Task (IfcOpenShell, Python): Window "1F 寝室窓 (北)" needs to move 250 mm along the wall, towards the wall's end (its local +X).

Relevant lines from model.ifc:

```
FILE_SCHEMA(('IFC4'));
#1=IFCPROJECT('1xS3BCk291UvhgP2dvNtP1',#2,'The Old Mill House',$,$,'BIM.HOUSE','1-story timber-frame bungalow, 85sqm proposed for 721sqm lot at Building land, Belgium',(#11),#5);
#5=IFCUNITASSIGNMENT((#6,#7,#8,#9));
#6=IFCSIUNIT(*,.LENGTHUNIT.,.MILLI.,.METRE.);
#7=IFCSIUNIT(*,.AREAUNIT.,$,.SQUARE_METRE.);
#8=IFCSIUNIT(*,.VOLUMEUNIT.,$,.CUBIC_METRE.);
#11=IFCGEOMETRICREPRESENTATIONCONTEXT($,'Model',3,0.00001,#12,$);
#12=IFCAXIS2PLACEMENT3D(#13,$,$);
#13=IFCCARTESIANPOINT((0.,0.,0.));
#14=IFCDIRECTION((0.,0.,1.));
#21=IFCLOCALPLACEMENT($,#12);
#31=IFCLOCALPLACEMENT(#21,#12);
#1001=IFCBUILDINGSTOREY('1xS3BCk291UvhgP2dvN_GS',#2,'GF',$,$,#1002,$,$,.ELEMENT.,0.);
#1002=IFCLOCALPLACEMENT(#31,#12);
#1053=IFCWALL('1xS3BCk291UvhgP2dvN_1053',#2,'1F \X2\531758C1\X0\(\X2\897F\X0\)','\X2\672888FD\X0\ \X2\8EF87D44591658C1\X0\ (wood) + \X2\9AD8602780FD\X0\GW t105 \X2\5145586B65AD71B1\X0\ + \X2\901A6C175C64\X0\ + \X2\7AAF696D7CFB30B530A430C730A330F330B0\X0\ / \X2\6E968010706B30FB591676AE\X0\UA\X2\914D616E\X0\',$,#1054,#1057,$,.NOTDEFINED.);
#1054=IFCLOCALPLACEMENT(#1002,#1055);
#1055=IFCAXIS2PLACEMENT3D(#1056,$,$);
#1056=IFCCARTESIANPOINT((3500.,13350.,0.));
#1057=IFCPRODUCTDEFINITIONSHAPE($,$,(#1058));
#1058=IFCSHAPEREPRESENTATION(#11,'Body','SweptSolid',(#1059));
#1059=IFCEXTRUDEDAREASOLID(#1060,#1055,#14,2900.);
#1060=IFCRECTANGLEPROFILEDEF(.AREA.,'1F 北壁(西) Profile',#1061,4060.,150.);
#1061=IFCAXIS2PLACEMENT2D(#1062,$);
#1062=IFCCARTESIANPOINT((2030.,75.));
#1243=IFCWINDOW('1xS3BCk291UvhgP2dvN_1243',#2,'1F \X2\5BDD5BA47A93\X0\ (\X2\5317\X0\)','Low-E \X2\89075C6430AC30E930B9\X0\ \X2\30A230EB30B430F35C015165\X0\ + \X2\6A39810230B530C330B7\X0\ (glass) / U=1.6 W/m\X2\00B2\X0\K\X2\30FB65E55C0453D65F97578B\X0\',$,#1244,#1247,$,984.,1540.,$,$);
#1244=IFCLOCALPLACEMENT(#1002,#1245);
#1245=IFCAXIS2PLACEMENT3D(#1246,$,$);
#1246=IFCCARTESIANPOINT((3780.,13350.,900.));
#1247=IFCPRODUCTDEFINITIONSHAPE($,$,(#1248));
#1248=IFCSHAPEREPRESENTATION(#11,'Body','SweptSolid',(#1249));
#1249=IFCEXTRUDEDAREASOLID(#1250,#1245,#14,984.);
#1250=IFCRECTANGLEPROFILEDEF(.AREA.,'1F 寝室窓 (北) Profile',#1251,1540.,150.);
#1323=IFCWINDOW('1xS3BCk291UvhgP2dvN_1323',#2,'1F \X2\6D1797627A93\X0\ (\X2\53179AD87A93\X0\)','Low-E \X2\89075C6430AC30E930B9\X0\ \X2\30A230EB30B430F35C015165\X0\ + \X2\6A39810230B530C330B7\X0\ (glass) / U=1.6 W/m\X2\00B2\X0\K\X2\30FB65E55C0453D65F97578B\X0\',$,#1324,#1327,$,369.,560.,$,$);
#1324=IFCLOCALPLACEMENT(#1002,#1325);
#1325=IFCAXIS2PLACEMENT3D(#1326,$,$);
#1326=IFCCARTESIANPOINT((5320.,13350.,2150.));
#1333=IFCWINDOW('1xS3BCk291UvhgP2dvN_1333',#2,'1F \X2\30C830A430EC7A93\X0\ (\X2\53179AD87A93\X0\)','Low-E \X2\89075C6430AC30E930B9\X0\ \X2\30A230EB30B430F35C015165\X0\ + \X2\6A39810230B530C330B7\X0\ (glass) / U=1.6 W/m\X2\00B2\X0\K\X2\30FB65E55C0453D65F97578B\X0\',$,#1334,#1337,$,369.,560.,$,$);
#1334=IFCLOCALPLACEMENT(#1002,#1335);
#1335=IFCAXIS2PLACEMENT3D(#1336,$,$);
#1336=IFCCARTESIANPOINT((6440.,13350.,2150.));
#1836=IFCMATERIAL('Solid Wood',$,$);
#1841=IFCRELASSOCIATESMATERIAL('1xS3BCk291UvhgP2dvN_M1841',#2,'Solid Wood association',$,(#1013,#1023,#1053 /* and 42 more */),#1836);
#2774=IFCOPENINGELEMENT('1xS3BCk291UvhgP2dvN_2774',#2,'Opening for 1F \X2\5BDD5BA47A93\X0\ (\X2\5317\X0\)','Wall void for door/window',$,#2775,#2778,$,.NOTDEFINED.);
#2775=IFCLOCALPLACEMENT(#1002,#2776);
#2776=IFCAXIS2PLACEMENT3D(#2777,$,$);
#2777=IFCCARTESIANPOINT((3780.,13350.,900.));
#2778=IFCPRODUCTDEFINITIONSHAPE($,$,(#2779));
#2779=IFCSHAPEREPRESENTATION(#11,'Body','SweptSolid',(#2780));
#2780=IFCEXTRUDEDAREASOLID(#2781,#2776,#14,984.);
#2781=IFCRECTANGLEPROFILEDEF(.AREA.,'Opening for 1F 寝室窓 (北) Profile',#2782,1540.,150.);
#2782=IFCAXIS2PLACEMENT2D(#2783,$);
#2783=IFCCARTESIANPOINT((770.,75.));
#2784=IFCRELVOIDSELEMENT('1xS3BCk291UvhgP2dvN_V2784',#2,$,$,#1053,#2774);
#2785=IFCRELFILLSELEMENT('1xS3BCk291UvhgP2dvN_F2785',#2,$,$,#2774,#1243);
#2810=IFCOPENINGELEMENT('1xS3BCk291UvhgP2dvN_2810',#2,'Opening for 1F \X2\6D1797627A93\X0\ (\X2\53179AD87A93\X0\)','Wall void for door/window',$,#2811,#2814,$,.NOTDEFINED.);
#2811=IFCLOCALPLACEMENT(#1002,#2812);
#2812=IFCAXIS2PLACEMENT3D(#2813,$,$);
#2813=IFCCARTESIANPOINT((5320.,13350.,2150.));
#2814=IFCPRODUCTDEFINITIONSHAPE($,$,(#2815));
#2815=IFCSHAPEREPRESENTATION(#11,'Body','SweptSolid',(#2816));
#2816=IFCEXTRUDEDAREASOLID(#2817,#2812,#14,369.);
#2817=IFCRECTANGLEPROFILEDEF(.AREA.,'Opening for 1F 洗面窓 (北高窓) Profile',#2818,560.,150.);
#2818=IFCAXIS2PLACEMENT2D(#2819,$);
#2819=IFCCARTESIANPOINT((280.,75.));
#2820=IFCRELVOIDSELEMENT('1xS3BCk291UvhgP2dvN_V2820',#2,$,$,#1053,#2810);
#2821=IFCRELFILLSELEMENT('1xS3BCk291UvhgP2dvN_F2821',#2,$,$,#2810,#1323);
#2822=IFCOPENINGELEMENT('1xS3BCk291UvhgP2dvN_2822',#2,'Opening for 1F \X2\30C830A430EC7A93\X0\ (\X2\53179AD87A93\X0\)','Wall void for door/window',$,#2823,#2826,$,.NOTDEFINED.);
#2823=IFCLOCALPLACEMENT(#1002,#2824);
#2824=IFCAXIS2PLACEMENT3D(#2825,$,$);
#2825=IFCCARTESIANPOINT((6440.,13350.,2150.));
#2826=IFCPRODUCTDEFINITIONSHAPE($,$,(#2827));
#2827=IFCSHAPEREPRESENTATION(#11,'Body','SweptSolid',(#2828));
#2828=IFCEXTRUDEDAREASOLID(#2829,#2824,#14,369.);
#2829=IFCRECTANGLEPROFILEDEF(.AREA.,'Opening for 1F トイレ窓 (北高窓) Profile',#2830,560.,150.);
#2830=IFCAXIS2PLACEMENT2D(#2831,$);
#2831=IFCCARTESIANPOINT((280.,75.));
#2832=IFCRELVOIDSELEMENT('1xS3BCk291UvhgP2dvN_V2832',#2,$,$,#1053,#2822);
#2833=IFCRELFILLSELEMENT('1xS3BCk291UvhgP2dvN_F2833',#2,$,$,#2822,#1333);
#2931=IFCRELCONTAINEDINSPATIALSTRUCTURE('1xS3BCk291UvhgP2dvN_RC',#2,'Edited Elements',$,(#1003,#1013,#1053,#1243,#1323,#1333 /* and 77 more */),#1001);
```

```python
import ifcopenshell
import ifcopenshell.api.geometry
import ifcopenshell.util.placement
import ifcopenshell.util.unit

model = ifcopenshell.open("model.ifc")
unit_scale = ifcopenshell.util.unit.calculate_unit_scale(model)

window = model.by_id(1243)
opening = window.FillsVoids[0].RelatingOpeningElement
wall = opening.VoidsElements[0].RelatingBuildingElement

wall_matrix = ifcopenshell.util.placement.get_local_placement(wall.ObjectPlacement)
shift = wall_matrix[:3, 0] * 0.25 / unit_scale
before = ifcopenshell.util.placement.get_local_placement(window.ObjectPlacement)[:3, 3].copy()

# The window is not placed relative to its opening, so move both.
for product in (opening, window):
    matrix = ifcopenshell.util.placement.get_local_placement(product.ObjectPlacement)
    matrix[:3, 3] += shift
    ifcopenshell.api.geometry.edit_object_placement(model, product=product, matrix=matrix, is_si=False)

after = ifcopenshell.util.placement.get_local_placement(window.ObjectPlacement)[:3, 3]
print("window moved by", (after - before).round(3) + 0.0)

model.write("model_v2.ifc")
```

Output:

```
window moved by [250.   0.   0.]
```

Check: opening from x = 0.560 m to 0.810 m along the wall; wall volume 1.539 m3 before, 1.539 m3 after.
